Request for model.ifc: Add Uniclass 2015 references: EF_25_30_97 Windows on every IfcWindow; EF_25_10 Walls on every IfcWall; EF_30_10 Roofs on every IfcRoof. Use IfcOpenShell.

First a look at what the model holds.

```python
import ifcopenshell

model = ifcopenshell.open("model.ifc")
print(model.schema)
print("classifications:", [c.Name for c in model.by_type("IfcClassification")])
for ifc_class in ("IfcDoor", "IfcRoof", "IfcStair", "IfcWall", "IfcWindow"):
    print(ifc_class, len(model.by_type(ifc_class)))
```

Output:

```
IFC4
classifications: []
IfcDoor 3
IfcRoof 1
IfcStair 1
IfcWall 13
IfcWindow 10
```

```python
import ifcopenshell
import ifcopenshell.api.classification

model = ifcopenshell.open("model.ifc")

system = ifcopenshell.api.classification.add_classification(model, classification="Uniclass 2015")

codes = {
    "IfcWindow": ("EF_25_30_97", "Windows"),
    "IfcWall": ("EF_25_10", "Walls"),
    "IfcRoof": ("EF_30_10", "Roofs"),
}
for ifc_class, (code, name) in codes.items():
    products = model.by_type(ifc_class)
    ifcopenshell.api.classification.add_reference(
        model, products=products, classification=system, identification=code, name=name
    )
    print(code, len(products))

model.write("model_v2.ifc")
```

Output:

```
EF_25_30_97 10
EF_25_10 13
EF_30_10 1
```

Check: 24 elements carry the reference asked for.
